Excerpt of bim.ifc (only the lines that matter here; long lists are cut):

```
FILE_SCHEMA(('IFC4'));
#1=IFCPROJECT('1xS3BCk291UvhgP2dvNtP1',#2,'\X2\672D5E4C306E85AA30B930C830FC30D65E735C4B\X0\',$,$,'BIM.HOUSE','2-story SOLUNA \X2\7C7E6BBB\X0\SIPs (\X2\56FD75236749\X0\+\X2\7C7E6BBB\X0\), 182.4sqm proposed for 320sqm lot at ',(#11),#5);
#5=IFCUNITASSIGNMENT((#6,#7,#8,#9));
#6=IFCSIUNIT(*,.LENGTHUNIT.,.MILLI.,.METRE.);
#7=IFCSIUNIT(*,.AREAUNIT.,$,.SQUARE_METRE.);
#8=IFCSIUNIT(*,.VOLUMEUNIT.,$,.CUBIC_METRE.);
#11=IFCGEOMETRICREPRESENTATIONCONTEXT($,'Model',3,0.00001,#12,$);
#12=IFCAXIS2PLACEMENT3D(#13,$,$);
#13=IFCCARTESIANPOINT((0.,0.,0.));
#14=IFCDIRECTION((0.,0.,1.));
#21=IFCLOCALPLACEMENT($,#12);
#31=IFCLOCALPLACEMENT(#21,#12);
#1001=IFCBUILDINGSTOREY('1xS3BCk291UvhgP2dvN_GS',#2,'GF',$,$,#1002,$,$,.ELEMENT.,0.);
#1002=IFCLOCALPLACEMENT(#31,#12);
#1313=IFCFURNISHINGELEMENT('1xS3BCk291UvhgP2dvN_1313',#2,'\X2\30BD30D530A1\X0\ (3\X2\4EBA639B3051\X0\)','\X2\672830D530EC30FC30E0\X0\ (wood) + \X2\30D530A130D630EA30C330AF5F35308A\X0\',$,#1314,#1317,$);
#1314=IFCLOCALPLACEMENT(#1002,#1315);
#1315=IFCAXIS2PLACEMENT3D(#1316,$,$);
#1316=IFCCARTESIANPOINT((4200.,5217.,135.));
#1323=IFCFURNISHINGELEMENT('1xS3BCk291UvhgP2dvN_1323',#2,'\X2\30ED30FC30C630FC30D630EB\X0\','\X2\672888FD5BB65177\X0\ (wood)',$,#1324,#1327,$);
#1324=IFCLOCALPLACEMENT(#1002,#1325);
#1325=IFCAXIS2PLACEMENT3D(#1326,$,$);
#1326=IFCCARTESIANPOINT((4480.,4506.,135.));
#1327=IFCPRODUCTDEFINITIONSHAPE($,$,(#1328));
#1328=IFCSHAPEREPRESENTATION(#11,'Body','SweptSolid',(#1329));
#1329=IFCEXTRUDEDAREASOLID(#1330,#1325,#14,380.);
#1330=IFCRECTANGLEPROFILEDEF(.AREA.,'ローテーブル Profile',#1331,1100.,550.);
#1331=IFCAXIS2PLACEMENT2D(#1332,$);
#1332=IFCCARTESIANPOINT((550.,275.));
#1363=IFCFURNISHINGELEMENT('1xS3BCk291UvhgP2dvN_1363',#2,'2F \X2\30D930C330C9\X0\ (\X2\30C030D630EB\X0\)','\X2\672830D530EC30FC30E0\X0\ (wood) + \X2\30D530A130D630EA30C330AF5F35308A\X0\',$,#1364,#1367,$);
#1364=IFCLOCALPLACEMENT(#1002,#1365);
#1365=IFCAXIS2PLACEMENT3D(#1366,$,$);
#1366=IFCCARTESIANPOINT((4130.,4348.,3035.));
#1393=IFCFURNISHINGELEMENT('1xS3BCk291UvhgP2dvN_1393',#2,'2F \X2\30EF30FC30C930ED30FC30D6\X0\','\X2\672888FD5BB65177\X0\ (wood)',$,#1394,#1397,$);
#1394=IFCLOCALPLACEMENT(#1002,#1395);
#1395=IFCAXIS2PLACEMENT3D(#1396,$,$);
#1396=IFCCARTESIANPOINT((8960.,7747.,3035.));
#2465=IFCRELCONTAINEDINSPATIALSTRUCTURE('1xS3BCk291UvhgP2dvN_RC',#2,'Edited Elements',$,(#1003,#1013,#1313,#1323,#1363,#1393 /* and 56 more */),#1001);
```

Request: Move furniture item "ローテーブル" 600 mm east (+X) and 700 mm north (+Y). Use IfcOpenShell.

```python
import ifcopenshell
import ifcopenshell.api.geometry
import ifcopenshell.util.placement
import ifcopenshell.util.unit

model = ifcopenshell.open("bim.ifc")
unit_scale = ifcopenshell.util.unit.calculate_unit_scale(model)

item = model.by_guid("1xS3BCk291UvhgP2dvN_1323")
matrix = ifcopenshell.util.placement.get_local_placement(item.ObjectPlacement)
matrix[0, 3] += 0.6 / unit_scale
matrix[1, 3] += 0.7 / unit_scale
ifcopenshell.api.geometry.edit_object_placement(model, product=item, matrix=matrix, is_si=False)

print(ifcopenshell.util.placement.get_local_placement(item.ObjectPlacement).round(3) + 0.0)

model.write("bim-out.ifc")
```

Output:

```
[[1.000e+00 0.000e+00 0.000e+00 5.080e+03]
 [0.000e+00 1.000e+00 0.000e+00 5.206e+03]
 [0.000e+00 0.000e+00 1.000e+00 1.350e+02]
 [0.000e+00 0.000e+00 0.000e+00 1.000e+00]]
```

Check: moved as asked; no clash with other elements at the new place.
